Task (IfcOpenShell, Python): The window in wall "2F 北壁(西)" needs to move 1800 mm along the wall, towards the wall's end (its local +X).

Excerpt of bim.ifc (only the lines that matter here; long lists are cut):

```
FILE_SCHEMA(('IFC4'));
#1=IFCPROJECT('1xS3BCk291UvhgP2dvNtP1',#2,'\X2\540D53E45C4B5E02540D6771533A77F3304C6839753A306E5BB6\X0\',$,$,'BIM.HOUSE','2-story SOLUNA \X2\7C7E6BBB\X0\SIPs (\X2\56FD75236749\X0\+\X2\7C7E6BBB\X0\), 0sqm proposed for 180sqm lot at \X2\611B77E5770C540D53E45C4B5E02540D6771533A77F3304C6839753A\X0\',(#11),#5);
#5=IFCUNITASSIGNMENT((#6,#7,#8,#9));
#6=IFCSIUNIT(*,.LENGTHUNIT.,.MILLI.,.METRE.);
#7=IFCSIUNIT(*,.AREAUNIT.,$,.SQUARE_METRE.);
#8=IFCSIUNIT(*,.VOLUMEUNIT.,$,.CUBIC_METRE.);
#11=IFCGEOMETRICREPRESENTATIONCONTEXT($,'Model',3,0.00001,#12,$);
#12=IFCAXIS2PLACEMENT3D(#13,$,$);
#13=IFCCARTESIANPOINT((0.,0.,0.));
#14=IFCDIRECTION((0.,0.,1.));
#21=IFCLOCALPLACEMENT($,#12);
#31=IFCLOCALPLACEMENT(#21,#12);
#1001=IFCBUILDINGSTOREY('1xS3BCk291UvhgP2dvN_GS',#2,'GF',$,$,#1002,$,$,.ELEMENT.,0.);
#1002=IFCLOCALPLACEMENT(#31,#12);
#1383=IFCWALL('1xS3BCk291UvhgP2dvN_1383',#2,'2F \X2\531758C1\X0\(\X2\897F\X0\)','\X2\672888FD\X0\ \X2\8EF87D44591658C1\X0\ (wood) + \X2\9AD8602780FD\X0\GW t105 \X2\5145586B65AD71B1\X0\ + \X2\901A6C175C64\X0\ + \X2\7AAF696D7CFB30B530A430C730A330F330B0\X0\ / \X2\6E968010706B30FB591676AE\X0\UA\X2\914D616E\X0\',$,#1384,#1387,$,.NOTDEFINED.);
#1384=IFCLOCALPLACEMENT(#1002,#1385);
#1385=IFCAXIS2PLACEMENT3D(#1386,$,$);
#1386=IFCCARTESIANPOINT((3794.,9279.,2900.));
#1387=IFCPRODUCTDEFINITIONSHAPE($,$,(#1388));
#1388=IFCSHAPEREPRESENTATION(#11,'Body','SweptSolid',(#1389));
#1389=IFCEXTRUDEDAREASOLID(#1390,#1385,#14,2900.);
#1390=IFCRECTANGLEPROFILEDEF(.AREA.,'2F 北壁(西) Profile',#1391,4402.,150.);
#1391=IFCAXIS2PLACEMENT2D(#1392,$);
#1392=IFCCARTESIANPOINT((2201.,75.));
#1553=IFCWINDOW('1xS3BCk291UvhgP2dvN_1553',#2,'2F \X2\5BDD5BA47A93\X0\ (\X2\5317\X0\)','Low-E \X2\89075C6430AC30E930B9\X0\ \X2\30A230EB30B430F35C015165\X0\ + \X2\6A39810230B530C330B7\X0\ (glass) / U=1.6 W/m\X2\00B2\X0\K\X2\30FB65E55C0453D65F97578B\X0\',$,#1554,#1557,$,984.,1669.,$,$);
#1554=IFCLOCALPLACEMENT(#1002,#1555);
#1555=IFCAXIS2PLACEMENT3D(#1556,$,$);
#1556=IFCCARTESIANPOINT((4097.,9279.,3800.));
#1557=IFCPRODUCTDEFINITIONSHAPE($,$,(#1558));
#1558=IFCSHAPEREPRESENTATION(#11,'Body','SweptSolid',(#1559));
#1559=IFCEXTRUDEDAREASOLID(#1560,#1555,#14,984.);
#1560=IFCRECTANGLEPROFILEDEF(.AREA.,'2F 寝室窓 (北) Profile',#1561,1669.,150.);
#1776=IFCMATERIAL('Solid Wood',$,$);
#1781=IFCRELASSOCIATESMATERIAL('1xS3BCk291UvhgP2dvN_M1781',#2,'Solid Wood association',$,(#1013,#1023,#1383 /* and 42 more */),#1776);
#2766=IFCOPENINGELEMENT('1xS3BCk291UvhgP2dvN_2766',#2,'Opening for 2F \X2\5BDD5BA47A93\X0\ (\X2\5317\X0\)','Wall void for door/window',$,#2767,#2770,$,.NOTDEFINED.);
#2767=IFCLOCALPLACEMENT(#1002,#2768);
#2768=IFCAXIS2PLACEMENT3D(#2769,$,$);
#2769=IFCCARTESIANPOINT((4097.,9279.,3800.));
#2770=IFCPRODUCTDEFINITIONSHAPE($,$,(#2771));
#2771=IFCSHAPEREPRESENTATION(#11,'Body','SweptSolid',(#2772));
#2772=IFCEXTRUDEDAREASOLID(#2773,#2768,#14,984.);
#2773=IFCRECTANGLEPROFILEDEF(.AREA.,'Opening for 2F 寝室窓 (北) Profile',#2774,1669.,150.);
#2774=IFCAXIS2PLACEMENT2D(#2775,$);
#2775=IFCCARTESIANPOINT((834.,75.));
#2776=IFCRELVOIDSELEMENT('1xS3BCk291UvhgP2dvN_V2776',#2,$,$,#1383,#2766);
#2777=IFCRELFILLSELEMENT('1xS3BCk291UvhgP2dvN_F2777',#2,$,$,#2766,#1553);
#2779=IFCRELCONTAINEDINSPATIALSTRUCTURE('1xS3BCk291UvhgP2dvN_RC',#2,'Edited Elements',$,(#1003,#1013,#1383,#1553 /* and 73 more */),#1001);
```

```python
import ifcopenshell
import ifcopenshell.api.geometry
import ifcopenshell.util.placement

model = ifcopenshell.open("bim.ifc")

window = model.by_id(1553)
opening = window.FillsVoids[0].RelatingOpeningElement
wall = opening.VoidsElements[0].RelatingBuildingElement

wall_matrix = ifcopenshell.util.placement.get_local_placement(wall.ObjectPlacement)
shift = wall_matrix[:3, 0] * 1800.0
before = ifcopenshell.util.placement.get_local_placement(window.ObjectPlacement)[:3, 3].copy()

# The window is not placed relative to its opening, so move both.
for product in (opening, window):
    matrix = ifcopenshell.util.placement.get_local_placement(product.ObjectPlacement)
    matrix[:3, 3] += shift
    ifcopenshell.api.geometry.edit_object_placement(model, product=product, matrix=matrix, is_si=False)

after = ifcopenshell.util.placement.get_local_placement(window.ObjectPlacement)[:3, 3]
print("window moved by", (after - before).round(3) + 0.0)

model.write("bim-out.ifc")
```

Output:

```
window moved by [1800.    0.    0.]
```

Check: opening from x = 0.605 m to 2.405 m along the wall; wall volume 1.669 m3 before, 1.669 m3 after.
